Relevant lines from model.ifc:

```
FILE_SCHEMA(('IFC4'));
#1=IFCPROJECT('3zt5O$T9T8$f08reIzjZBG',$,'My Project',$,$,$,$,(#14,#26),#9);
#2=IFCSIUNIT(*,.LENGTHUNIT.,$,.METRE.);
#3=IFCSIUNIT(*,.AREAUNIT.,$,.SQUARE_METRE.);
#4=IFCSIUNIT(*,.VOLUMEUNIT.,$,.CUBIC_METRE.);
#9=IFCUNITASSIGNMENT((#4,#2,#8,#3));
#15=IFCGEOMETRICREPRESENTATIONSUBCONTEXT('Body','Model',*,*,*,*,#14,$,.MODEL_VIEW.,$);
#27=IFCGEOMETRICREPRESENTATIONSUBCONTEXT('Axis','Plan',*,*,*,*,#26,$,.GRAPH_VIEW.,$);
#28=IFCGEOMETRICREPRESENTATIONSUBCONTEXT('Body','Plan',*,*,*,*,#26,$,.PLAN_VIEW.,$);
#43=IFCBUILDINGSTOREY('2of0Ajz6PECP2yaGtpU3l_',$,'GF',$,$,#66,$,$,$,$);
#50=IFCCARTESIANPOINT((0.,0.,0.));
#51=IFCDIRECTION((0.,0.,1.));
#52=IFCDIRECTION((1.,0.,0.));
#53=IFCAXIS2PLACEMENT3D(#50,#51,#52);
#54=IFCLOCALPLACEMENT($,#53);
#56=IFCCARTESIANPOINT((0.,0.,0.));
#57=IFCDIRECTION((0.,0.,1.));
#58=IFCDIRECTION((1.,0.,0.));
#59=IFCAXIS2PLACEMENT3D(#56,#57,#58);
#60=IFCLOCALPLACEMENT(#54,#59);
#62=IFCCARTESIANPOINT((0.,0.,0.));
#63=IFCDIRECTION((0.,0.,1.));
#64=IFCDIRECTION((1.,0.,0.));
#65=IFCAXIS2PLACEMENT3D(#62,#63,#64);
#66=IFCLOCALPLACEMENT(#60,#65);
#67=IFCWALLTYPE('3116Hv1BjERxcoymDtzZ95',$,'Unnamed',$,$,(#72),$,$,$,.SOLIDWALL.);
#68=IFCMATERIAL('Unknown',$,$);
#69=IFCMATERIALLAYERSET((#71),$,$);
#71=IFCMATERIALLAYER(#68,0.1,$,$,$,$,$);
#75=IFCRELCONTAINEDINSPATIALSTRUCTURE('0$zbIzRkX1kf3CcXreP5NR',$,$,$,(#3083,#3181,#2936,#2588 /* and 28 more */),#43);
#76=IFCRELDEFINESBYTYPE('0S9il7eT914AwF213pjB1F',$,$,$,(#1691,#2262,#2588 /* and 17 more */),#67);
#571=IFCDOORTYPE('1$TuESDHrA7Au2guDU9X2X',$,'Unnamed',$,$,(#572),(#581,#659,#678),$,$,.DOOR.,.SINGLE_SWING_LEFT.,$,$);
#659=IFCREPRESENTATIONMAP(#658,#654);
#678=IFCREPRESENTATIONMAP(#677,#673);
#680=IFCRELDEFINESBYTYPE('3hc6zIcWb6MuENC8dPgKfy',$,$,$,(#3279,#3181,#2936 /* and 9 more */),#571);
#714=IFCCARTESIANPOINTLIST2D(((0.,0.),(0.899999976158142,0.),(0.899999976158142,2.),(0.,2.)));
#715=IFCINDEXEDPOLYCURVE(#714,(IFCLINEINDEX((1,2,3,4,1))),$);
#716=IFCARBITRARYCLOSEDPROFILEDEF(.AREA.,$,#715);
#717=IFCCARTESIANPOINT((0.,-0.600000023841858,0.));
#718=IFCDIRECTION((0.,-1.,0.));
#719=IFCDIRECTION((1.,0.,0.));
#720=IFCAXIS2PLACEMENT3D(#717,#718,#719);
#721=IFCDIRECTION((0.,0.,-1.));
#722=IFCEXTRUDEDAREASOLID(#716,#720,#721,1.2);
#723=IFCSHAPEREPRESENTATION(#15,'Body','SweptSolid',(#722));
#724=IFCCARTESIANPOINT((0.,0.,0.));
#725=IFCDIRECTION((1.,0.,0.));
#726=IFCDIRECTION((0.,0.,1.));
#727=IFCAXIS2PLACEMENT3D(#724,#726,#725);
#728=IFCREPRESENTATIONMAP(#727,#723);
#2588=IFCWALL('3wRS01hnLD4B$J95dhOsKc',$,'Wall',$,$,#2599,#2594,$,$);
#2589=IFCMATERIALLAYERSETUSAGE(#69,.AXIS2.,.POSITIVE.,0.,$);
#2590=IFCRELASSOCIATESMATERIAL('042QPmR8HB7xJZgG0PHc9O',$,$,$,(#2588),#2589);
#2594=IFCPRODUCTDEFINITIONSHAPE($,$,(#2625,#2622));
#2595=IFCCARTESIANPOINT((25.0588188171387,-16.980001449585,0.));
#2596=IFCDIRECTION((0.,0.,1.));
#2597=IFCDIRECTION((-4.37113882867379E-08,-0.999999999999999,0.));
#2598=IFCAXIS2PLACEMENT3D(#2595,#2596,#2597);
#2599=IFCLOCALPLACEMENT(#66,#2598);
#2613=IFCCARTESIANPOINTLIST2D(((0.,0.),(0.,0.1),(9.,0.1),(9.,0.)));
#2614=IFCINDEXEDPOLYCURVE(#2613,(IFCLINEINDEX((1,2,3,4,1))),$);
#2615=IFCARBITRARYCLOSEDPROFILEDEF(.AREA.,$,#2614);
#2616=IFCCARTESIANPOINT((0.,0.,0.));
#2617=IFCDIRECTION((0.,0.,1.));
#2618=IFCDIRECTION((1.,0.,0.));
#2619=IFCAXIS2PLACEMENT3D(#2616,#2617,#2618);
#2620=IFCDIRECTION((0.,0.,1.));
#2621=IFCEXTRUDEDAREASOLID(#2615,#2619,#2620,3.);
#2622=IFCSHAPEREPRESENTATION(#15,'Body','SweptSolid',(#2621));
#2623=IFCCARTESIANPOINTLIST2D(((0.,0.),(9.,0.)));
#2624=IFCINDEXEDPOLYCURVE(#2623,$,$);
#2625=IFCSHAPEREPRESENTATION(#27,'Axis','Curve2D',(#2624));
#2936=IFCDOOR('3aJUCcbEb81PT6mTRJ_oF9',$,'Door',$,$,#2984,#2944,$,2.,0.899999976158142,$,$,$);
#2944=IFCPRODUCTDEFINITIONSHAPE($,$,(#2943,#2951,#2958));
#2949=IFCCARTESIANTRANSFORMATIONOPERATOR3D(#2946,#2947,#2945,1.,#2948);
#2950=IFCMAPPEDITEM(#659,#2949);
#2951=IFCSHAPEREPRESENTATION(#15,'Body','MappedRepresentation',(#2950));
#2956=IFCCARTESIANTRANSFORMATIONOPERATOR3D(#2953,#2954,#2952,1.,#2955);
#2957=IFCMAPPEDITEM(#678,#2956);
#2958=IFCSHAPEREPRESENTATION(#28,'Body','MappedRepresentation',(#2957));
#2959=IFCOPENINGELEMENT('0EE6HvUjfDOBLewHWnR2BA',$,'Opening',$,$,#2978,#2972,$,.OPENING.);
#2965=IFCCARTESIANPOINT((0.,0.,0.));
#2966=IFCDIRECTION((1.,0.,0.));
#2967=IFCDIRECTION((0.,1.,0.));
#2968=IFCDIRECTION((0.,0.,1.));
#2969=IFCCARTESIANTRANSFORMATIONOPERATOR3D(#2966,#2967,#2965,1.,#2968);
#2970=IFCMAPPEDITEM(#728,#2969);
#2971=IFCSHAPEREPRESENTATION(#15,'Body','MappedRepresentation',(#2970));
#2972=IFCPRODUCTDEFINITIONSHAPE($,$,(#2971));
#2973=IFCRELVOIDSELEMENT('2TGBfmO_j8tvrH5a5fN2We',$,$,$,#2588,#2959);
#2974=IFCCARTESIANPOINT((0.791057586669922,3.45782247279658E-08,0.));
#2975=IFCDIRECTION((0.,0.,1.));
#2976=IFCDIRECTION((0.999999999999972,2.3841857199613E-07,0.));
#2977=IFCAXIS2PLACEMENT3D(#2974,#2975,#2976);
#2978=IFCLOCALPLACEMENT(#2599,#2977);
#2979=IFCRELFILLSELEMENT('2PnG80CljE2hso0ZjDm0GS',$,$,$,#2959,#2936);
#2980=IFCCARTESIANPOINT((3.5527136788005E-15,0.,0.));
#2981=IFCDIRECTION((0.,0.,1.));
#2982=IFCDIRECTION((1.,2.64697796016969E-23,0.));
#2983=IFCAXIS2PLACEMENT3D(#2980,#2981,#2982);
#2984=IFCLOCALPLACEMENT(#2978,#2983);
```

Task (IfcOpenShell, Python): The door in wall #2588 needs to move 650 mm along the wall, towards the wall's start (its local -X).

```python
import ifcopenshell
import ifcopenshell.api.geometry
import ifcopenshell.util.placement

model = ifcopenshell.open("model.ifc")

door = model.by_guid("3aJUCcbEb81PT6mTRJ_oF9")
opening = door.FillsVoids[0].RelatingOpeningElement
wall = opening.VoidsElements[0].RelatingBuildingElement

wall_matrix = ifcopenshell.util.placement.get_local_placement(wall.ObjectPlacement)
shift = wall_matrix[:3, 0] * -0.65
before = ifcopenshell.util.placement.get_local_placement(door.ObjectPlacement)[:3, 3].copy()

# The door is placed relative to its opening, so it follows when the opening moves.
matrix = ifcopenshell.util.placement.get_local_placement(opening.ObjectPlacement)
matrix[:3, 3] += shift
ifcopenshell.api.geometry.edit_object_placement(
    model, product=opening, matrix=matrix, is_si=False, should_transform_children=True
)

after = ifcopenshell.util.placement.get_local_placement(door.ObjectPlacement)[:3, 3]
print("door moved by", (after - before).round(3) + 0.0)

model.write("model_v2.ifc")
```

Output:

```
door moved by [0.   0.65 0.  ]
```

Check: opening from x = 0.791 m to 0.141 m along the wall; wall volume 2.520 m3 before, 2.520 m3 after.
